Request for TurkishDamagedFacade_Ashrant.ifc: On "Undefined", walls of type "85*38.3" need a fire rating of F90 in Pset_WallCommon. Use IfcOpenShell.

First a look at what the model holds.

```python
import ifcopenshell
import ifcopenshell.util.element

model = ifcopenshell.open("TurkishDamagedFacade_Ashrant.ifc")
print(model.schema)
storey = next(s for s in model.by_type("IfcBuildingStorey") if s.Name == "Undefined")
walls = [e for e in ifcopenshell.util.element.get_decomposition(storey) if e.is_a("IfcWall")]
seen = {}
for e in walls:
    element_type = ifcopenshell.util.element.get_type(e)
    key = (element_type.Name if element_type != e and element_type else None, ifcopenshell.util.element.get_pset(e, "Pset_WallCommon", "FireRating"))
    seen[key] = seen.get(key, 0) + 1
for (name, value), count in sorted(seen.items(), key=str):
    print(count, "x", name, "|", value)
```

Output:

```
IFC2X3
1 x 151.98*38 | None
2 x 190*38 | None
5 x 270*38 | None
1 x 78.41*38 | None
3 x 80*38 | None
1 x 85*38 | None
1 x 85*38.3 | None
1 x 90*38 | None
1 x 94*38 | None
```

```python
import ifcopenshell
import ifcopenshell.api.pset
import ifcopenshell.util.element

model = ifcopenshell.open("TurkishDamagedFacade_Ashrant.ifc")

storey = next(s for s in model.by_type("IfcBuildingStorey") if s.Name == "Undefined")
walls = [e for e in ifcopenshell.util.element.get_decomposition(storey) if e.is_a("IfcWall")]

count = 0
for e in walls:
    element_type = ifcopenshell.util.element.get_type(e)
    if element_type in (None, e) or element_type.Name != "85*38.3":
        continue
    # add_pset returns the element's existing set when there is one.
    pset = ifcopenshell.api.pset.add_pset(model, product=e, name="Pset_WallCommon")
    ifcopenshell.api.pset.edit_pset(model, pset=pset, properties={"FireRating": "F90"})
    count += 1

print(count, "walls updated")

model.write("TurkishDamagedFacade_Ashrant_edited.ifc")
```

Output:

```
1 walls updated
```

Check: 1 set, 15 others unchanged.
